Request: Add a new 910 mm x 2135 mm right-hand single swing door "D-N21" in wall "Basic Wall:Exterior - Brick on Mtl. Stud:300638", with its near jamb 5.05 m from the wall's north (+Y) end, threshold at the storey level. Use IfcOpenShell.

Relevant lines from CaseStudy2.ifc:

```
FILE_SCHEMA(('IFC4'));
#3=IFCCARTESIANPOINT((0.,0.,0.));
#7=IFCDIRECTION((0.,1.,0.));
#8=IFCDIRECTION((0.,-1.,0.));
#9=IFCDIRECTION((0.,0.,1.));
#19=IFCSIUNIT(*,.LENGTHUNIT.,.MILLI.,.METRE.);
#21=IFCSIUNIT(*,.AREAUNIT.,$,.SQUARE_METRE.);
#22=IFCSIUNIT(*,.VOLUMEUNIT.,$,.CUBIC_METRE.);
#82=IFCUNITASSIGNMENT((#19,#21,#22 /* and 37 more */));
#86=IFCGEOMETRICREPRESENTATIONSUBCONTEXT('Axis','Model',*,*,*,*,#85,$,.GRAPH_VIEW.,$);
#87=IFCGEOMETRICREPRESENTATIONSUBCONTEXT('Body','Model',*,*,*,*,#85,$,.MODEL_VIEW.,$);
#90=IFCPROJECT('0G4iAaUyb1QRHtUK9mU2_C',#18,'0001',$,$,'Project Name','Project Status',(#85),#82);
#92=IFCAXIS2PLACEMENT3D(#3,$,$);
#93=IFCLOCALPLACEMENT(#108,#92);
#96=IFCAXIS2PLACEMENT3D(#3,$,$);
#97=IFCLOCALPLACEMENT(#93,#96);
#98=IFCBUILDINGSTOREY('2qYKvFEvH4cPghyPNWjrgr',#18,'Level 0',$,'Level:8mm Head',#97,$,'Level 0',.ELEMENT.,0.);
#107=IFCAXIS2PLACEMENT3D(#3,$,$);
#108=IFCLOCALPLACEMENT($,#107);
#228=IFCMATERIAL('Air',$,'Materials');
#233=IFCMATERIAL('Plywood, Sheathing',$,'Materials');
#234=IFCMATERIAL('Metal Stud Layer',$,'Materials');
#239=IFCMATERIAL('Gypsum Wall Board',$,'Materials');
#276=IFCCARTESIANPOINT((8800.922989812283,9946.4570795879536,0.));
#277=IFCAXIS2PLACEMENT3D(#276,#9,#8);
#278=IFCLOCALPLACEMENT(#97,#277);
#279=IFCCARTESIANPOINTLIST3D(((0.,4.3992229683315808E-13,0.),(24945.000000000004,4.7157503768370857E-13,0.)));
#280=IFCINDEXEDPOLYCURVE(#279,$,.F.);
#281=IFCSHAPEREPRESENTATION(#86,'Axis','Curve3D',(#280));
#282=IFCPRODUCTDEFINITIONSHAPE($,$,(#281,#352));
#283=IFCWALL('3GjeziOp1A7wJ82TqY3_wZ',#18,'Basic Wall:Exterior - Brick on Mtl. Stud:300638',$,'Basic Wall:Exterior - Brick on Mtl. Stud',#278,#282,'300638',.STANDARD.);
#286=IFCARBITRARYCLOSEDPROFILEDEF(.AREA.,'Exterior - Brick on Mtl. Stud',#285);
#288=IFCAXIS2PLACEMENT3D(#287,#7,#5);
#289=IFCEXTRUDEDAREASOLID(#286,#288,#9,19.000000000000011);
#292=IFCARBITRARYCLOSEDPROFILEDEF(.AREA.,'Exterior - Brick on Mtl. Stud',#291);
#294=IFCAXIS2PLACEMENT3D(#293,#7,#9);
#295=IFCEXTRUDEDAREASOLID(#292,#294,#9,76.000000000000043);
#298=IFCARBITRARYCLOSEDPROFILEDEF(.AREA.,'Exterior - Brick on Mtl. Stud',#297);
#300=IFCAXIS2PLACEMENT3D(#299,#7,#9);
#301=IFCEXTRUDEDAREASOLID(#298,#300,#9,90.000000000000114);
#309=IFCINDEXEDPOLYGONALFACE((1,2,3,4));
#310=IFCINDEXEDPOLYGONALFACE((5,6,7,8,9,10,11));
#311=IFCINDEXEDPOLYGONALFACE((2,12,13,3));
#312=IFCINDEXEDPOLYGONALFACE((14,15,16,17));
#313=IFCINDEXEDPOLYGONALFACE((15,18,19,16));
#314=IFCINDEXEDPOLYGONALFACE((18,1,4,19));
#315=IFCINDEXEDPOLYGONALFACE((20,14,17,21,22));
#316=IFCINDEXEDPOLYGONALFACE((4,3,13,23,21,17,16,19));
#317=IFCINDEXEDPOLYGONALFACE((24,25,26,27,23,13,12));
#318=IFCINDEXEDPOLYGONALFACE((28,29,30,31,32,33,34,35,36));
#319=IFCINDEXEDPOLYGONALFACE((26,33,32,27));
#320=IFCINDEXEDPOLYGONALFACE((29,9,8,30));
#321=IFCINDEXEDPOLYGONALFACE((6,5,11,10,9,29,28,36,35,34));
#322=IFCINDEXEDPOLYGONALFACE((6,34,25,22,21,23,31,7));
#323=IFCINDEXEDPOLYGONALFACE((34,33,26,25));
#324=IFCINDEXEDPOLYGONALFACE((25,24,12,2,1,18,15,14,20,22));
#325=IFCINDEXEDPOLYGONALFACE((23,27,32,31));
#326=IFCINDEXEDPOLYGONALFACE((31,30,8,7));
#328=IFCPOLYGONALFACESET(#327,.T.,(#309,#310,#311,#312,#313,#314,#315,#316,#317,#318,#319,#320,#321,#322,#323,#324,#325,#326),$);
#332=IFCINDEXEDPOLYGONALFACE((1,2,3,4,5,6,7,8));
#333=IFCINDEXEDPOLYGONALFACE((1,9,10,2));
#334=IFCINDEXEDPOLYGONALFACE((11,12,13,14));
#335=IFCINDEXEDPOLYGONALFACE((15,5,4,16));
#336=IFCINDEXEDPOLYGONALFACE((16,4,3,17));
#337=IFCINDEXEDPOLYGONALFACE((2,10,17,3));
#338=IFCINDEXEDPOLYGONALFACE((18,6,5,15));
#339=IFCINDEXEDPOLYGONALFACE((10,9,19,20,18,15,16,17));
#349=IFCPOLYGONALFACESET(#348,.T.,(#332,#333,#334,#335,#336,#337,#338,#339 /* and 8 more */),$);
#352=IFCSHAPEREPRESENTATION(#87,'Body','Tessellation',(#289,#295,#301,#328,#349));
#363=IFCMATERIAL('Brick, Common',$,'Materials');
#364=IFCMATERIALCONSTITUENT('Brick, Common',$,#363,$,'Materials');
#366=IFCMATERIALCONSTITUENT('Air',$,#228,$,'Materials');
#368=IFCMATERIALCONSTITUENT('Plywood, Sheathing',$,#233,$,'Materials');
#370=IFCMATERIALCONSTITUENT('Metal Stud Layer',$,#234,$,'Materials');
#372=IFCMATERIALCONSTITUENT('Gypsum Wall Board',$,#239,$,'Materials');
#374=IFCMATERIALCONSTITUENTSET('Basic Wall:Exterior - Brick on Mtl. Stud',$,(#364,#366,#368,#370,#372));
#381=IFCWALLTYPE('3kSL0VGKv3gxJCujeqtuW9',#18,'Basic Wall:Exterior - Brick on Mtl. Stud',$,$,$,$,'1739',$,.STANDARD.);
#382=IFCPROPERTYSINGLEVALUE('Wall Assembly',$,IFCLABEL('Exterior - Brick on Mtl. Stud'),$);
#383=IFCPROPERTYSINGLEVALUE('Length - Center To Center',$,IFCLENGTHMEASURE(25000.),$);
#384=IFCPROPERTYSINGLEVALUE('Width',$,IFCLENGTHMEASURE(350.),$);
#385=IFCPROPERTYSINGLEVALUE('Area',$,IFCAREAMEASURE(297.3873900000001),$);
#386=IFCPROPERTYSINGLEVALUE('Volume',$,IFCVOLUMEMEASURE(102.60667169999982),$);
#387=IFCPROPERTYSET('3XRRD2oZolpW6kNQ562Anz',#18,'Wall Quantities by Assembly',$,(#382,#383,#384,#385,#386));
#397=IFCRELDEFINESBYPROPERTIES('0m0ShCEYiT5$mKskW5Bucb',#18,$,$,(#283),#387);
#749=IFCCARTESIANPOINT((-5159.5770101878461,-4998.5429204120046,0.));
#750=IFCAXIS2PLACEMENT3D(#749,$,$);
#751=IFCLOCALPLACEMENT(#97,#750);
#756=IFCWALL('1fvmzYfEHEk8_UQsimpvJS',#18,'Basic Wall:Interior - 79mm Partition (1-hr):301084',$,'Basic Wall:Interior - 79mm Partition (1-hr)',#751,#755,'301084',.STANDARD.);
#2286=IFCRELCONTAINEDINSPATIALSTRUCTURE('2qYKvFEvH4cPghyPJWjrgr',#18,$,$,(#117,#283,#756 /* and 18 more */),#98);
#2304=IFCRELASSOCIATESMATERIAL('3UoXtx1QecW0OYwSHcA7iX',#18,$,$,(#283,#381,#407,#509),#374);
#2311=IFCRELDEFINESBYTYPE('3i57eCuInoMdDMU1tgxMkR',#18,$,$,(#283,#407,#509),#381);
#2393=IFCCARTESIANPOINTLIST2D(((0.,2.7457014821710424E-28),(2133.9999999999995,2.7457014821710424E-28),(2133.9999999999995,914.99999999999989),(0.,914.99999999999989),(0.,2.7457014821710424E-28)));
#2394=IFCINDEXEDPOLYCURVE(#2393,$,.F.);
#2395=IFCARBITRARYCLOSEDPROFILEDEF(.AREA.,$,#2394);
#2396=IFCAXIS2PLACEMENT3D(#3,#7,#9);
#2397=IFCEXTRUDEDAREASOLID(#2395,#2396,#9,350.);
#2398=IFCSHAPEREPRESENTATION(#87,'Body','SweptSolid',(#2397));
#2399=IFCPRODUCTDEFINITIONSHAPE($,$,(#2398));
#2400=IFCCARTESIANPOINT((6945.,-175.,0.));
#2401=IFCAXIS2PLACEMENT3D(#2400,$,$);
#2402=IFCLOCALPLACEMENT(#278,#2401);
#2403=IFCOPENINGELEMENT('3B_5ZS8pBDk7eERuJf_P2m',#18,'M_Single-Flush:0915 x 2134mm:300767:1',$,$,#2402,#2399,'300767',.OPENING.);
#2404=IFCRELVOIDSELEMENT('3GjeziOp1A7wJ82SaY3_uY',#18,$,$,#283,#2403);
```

```python
import numpy as np
import ifcopenshell
import ifcopenshell.api.feature
import ifcopenshell.api.geometry
import ifcopenshell.api.pset
import ifcopenshell.api.root
import ifcopenshell.api.spatial
import ifcopenshell.geom
import ifcopenshell.util.element
import ifcopenshell.util.placement
import ifcopenshell.util.representation
import ifcopenshell.util.shape
import ifcopenshell.util.unit

model = ifcopenshell.open("CaseStudy2.ifc")
unit_scale = ifcopenshell.util.unit.calculate_unit_scale(model)
area_scale = ifcopenshell.util.unit.calculate_unit_scale(model, "AREAUNIT")
volume_scale = ifcopenshell.util.unit.calculate_unit_scale(model, "VOLUMEUNIT")
settings = ifcopenshell.geom.settings()


def volume(element):
    """Net volume in cubic metres, openings subtracted."""
    shape = ifcopenshell.geom.create_shape(settings, element)
    return ifcopenshell.util.shape.get_volume(shape.geometry)


wall = model.by_guid("3GjeziOp1A7wJ82TqY3_wZ")
storey = ifcopenshell.util.element.get_container(wall, ifc_class="IfcBuildingStorey")
context = ifcopenshell.util.representation.get_context(model, "Model", "Body", "MODEL_VIEW")
before = volume(wall)

width, height, from_end, sill = 0.91, 2.135, 5.05, 0.0  # metres

# The wall runs along its own X axis, and the end named is its -X end.
wall_shape = ifcopenshell.geom.create_shape(settings, wall)
x, y, z = ifcopenshell.util.shape.get_vertices(wall_shape.geometry).T
start = x.min() + from_end
face, thickness = float(y.min()), float(y.max() - y.min())
wall_matrix = ifcopenshell.util.placement.get_local_placement(wall.ObjectPlacement)
level = ifcopenshell.util.placement.get_local_placement(storey.ObjectPlacement)[2, 3]


def in_wall(x, y):
    """Placement at x, y metres in the wall's axes, at sill height."""
    matrix = wall_matrix.copy()
    matrix[:, 3] = wall_matrix @ np.array([x / unit_scale, y / unit_scale, 0.0, 1.0])
    matrix[2, 3] = level + sill / unit_scale
    return matrix


# Opening: a box that overshoots both wall faces by 50 mm.
opening = ifcopenshell.api.root.create_entity(model, ifc_class="IfcOpeningElement", predefined_type="OPENING")
box = ifcopenshell.api.geometry.add_wall_representation(
    model, context=context, length=width, height=height, thickness=thickness + 0.1
)
ifcopenshell.api.geometry.assign_representation(model, product=opening, representation=box)
ifcopenshell.api.geometry.edit_object_placement(model, product=opening, matrix=in_wall(start, face - 0.05), is_si=False)
ifcopenshell.api.feature.add_feature(model, feature=opening, element=wall)

door = ifcopenshell.api.root.create_entity(model, ifc_class="IfcDoor", name="D-N21", predefined_type="DOOR")
door.OverallWidth, door.OverallHeight = width / unit_scale, height / unit_scale
door.OperationType = "SINGLE_SWING_RIGHT"
body = ifcopenshell.api.geometry.add_door_representation(
    model,
    context=context,
    overall_width=door.OverallWidth,
    overall_height=door.OverallHeight,
    operation_type="SINGLE_SWING_RIGHT",
    lining_properties={"LiningDepth": thickness / unit_scale, "ThresholdDepth": thickness / unit_scale},
)
ifcopenshell.api.geometry.assign_representation(model, product=door, representation=body)
ifcopenshell.api.spatial.assign_container(model, products=[door], relating_structure=storey)
ifcopenshell.api.feature.add_filling(model, opening=opening, element=door)

# The lining spans the wall, so the door starts at the wall face.
ifcopenshell.api.geometry.edit_object_placement(model, product=door, matrix=in_wall(start, face), is_si=False)

after = volume(wall)

# Update the wall's stored quantities.
pset = model.by_id(ifcopenshell.util.element.get_pset(wall, "Wall Quantities by Assembly", should_inherit=False)["id"])
ifcopenshell.api.pset.edit_pset(model, pset=pset, properties={
    "Area": model.create_entity("IfcAreaMeasure", after / thickness / area_scale),
    "Volume": model.create_entity("IfcVolumeMeasure", after / volume_scale),
})

print(f"wall volume {before:.3f} -> {after:.3f} m3")

model.write("CaseStudy2_v2.ifc")
```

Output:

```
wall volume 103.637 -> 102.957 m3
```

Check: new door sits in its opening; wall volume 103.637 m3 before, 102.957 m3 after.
